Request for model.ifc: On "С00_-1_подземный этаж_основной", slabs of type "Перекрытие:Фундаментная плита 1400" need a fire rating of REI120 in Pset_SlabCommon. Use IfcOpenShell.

First a look at what the model holds.

```python
import ifcopenshell
import ifcopenshell.util.element

model = ifcopenshell.open("model.ifc")
print(model.schema)
storey = next(s for s in model.by_type("IfcBuildingStorey") if s.Name == "С00_-1_подземный этаж_основной")
slabs = [e for e in ifcopenshell.util.element.get_decomposition(storey) if e.is_a("IfcSlab")]
seen = {}
for e in slabs:
    element_type = ifcopenshell.util.element.get_type(e)
    key = (element_type.Name if element_type != e and element_type else None, ifcopenshell.util.element.get_pset(e, "Pset_SlabCommon", "FireRating"))
    seen[key] = seen.get(key, 0) + 1
for (name, value), count in sorted(seen.items(), key=str):
    print(count, "x", name, "|", value)
```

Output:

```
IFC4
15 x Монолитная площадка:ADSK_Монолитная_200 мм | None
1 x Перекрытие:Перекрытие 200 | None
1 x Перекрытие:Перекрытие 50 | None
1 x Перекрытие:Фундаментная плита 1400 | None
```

```python
import ifcopenshell
import ifcopenshell.api.pset
import ifcopenshell.util.element

model = ifcopenshell.open("model.ifc")

storey = next(s for s in model.by_type("IfcBuildingStorey") if s.Name == "С00_-1_подземный этаж_основной")
slabs = [e for e in ifcopenshell.util.element.get_decomposition(storey) if e.is_a("IfcSlab")]

count = 0
for e in slabs:
    element_type = ifcopenshell.util.element.get_type(e)
    if element_type in (None, e) or element_type.Name != "Перекрытие:Фундаментная плита 1400":
        continue
    # add_pset returns the element's existing set when there is one.
    pset = ifcopenshell.api.pset.add_pset(model, product=e, name="Pset_SlabCommon")
    ifcopenshell.api.pset.edit_pset(model, pset=pset, properties={"FireRating": "REI120"})
    count += 1

print(count, "slabs updated")

model.write("model_rev.ifc")
```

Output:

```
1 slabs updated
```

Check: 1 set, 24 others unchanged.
